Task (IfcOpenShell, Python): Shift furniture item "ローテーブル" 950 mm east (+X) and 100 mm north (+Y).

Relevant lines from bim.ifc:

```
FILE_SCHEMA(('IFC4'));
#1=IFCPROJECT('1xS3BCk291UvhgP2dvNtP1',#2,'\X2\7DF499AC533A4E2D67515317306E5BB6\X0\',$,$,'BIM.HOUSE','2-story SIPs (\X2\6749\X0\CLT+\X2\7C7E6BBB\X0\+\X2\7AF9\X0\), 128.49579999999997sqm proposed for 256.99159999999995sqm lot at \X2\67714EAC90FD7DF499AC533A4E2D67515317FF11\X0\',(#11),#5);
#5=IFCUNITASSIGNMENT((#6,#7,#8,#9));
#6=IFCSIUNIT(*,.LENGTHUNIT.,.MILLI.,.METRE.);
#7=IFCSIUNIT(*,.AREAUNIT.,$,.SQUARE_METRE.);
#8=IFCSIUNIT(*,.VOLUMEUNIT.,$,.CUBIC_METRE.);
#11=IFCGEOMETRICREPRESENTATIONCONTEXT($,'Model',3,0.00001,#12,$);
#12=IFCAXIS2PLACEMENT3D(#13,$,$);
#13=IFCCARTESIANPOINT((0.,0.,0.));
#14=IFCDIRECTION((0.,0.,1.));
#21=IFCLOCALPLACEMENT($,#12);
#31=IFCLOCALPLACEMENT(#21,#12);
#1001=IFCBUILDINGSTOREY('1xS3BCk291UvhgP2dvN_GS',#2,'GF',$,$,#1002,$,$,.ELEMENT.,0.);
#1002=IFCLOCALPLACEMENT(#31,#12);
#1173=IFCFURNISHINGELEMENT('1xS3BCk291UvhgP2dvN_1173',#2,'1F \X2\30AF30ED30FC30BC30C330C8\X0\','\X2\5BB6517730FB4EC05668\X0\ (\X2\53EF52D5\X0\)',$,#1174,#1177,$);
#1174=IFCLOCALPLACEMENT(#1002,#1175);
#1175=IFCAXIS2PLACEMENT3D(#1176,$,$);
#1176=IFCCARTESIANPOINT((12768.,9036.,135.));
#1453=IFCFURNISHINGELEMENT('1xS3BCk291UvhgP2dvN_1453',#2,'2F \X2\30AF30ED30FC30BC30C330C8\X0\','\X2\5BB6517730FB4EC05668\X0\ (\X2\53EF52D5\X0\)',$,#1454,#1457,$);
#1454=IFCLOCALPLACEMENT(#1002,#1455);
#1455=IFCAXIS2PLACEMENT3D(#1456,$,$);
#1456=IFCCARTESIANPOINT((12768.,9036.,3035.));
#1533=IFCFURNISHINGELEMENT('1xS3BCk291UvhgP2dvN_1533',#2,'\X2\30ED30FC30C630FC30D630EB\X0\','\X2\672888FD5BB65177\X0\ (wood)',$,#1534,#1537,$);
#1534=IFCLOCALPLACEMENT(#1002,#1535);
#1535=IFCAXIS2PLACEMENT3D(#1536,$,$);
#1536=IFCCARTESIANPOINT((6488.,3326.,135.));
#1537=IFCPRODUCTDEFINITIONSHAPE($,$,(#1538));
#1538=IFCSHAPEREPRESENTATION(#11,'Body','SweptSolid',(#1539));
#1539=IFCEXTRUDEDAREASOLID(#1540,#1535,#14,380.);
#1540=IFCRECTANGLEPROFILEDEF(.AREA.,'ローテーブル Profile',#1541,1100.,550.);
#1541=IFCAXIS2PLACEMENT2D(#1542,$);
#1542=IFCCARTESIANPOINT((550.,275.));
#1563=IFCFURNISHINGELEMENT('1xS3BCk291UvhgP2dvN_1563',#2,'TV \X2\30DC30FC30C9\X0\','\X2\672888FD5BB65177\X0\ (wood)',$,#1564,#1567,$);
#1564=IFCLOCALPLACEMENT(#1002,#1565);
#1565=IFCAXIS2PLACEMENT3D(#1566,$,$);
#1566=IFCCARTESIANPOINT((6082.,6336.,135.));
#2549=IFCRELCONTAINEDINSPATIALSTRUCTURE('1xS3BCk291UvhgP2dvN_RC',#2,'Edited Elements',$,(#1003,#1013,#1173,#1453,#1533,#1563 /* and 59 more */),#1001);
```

```python
import ifcopenshell
import ifcopenshell.api.geometry
import ifcopenshell.util.placement
import ifcopenshell.util.unit

model = ifcopenshell.open("bim.ifc")
unit_scale = ifcopenshell.util.unit.calculate_unit_scale(model)

item = model.by_guid("1xS3BCk291UvhgP2dvN_1533")
matrix = ifcopenshell.util.placement.get_local_placement(item.ObjectPlacement)
matrix[0, 3] += 0.95 / unit_scale
matrix[1, 3] += 0.1 / unit_scale
ifcopenshell.api.geometry.edit_object_placement(model, product=item, matrix=matrix, is_si=False)

print(ifcopenshell.util.placement.get_local_placement(item.ObjectPlacement).round(3) + 0.0)

model.write("bim_updated.ifc")
```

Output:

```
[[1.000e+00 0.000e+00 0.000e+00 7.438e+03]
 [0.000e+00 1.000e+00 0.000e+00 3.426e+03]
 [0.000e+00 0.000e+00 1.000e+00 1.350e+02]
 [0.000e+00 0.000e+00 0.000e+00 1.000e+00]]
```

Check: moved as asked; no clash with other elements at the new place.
